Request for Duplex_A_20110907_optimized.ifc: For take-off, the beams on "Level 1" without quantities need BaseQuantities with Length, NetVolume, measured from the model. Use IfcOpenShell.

First a look at what the model holds.

```python
import ifcopenshell
import ifcopenshell.util.element
import ifcopenshell.util.unit

model = ifcopenshell.open("Duplex_A_20110907_optimized.ifc")
print(model.schema)
for unit_type in ("LENGTHUNIT", "AREAUNIT", "VOLUMEUNIT"):
    print(unit_type, ifcopenshell.util.unit.calculate_unit_scale(model, unit_type))
storey = next(s for s in model.by_type("IfcBuildingStorey") if s.Name == "Level 1")
beams = [e for e in ifcopenshell.util.element.get_decomposition(storey) if e.is_a("IfcBeam")]
for e in sorted(beams, key=lambda e: e.id()):
    print(e.id(), e.is_a(), e.Name, list(ifcopenshell.util.element.get_psets(e, qtos_only=True)), sep=" | ")
```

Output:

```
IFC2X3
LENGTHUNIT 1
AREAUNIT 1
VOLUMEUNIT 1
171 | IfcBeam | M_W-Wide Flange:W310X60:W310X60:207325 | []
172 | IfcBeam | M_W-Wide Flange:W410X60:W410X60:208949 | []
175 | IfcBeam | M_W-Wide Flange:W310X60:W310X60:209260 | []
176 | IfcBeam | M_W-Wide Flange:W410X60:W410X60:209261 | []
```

```python
import ifcopenshell
import ifcopenshell.api.pset
import ifcopenshell.geom
import ifcopenshell.util.element
import ifcopenshell.util.shape
import ifcopenshell.util.unit

model = ifcopenshell.open("Duplex_A_20110907_optimized.ifc")
unit_scale = ifcopenshell.util.unit.calculate_unit_scale(model)
volume_scale = ifcopenshell.util.unit.calculate_unit_scale(model, "VOLUMEUNIT")
settings = ifcopenshell.geom.settings()

storey = next(s for s in model.by_type("IfcBuildingStorey") if s.Name == "Level 1")
beams = [e for e in ifcopenshell.util.element.get_decomposition(storey) if e.is_a("IfcBeam")]

for e in sorted(beams, key=lambda e: e.id()):
    if ifcopenshell.util.element.get_psets(e, qtos_only=True, should_inherit=False):
        continue
    # Geometry comes back in metres, in the element's own axes.
    shape = ifcopenshell.geom.create_shape(settings, e)
    values = {
        "Length": ifcopenshell.util.shape.get_max_xyz(shape.geometry) / unit_scale,
        "NetVolume": ifcopenshell.util.shape.get_volume(shape.geometry) / volume_scale,
    }
    qto = ifcopenshell.api.pset.add_qto(model, product=e, name="BaseQuantities")
    ifcopenshell.api.pset.edit_qto(model, qto=qto, properties=values)
    print(e.id(), {k: round(v, 3) for k, v in values.items()})

model.write("Duplex_A_20110907_optimized_rev.ifc")
```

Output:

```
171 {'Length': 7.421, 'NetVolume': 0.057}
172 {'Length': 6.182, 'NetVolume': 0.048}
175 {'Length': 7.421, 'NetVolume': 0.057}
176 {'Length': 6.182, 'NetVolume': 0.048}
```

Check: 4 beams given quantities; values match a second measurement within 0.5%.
